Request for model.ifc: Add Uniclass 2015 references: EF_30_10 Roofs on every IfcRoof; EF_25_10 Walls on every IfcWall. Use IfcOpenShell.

First a look at what the model holds.

```python
import ifcopenshell

model = ifcopenshell.open("model.ifc")
print(model.schema)
print("classifications:", [c.Name for c in model.by_type("IfcClassification")])
for ifc_class in ("IfcDoor", "IfcRoof", "IfcStair", "IfcWall", "IfcWindow"):
    print(ifc_class, len(model.by_type(ifc_class)))
```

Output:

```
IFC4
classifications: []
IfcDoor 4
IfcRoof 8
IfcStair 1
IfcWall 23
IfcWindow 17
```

```python
import ifcopenshell
import ifcopenshell.api.classification

model = ifcopenshell.open("model.ifc")

system = ifcopenshell.api.classification.add_classification(model, classification="Uniclass 2015")

codes = {
    "IfcRoof": ("EF_30_10", "Roofs"),
    "IfcWall": ("EF_25_10", "Walls"),
}
for ifc_class, (code, name) in codes.items():
    products = model.by_type(ifc_class)
    ifcopenshell.api.classification.add_reference(
        model, products=products, classification=system, identification=code, name=name
    )
    print(code, len(products))

model.write("model_rev.ifc")
```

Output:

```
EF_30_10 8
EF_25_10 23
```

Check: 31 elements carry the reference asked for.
